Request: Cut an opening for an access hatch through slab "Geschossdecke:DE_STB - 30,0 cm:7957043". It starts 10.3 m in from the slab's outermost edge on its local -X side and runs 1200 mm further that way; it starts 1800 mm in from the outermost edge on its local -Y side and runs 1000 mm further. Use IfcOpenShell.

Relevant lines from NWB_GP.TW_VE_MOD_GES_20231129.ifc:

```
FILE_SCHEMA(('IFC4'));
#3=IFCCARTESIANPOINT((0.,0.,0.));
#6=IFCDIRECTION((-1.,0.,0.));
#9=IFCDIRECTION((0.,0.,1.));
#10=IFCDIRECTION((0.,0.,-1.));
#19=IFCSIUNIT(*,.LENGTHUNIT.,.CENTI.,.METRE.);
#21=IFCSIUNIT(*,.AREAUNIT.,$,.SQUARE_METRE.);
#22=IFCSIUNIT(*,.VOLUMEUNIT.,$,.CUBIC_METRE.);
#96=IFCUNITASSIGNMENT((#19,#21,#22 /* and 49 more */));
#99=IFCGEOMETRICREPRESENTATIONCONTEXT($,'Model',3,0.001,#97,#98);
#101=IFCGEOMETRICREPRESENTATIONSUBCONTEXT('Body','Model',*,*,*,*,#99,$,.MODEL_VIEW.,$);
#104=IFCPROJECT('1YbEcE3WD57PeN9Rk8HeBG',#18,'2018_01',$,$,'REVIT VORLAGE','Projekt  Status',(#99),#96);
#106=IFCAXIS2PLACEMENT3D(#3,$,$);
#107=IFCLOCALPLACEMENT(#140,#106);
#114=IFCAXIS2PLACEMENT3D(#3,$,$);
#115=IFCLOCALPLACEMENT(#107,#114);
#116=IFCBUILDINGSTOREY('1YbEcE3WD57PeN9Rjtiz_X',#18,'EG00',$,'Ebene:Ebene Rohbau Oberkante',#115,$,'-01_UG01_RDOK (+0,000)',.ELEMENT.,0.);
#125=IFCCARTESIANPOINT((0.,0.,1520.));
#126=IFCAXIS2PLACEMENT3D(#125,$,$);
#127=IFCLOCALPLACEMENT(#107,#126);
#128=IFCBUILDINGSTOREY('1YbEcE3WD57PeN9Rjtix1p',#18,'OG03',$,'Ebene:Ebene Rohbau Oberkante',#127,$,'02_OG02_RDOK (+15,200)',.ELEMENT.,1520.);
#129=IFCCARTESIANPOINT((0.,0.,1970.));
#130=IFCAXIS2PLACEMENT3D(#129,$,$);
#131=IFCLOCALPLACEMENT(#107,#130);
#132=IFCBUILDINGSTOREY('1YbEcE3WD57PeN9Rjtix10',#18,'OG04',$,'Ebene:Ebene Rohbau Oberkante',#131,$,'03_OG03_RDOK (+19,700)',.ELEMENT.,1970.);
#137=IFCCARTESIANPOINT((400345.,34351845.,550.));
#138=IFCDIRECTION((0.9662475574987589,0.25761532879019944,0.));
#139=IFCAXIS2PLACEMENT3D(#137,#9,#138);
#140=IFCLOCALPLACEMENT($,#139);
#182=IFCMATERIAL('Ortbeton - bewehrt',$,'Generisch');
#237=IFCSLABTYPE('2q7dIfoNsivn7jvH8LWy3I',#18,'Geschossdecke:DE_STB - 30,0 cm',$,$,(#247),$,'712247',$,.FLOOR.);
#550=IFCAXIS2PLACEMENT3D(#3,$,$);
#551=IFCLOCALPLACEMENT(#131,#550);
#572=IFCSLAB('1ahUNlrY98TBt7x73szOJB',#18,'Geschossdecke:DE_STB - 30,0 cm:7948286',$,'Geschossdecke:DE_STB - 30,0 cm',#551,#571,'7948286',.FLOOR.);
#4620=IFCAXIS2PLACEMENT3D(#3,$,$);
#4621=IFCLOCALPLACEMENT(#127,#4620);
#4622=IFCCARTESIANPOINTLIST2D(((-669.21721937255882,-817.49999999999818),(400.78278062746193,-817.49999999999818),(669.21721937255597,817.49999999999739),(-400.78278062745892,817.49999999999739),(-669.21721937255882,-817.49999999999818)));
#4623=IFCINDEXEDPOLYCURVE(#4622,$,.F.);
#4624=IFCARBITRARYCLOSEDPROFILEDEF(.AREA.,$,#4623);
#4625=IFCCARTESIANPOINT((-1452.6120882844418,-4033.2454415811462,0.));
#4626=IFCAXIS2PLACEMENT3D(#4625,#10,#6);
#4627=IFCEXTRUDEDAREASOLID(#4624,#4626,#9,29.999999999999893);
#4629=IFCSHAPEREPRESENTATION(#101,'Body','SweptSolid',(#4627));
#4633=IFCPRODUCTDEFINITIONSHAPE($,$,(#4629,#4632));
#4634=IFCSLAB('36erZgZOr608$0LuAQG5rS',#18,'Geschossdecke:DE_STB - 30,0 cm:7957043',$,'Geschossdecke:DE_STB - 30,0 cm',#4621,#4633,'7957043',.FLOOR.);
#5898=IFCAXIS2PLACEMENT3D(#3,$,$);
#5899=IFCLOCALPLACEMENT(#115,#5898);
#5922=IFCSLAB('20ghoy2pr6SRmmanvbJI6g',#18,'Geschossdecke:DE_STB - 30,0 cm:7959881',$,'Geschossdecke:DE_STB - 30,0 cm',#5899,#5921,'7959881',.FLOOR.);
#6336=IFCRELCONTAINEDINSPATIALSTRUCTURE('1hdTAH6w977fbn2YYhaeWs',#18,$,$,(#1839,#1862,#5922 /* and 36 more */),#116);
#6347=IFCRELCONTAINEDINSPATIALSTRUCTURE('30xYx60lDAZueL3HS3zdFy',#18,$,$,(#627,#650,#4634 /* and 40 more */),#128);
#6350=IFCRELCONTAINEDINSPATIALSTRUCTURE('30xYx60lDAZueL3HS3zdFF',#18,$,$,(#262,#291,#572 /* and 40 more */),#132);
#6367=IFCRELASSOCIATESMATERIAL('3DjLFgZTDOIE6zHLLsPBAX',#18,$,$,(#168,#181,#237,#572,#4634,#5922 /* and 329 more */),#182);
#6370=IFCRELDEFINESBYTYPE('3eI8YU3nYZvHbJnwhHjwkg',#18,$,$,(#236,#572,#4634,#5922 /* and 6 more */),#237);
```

```python
import numpy as np
import ifcopenshell
import ifcopenshell.api.feature
import ifcopenshell.api.geometry
import ifcopenshell.api.root
import ifcopenshell.geom
import ifcopenshell.util.placement
import ifcopenshell.util.representation
import ifcopenshell.util.shape
import ifcopenshell.util.unit

model = ifcopenshell.open("NWB_GP.TW_VE_MOD_GES_20231129.ifc")
unit_scale = ifcopenshell.util.unit.calculate_unit_scale(model)
settings = ifcopenshell.geom.settings()


def volume(element):
    """Net volume in cubic metres, openings subtracted."""
    shape = ifcopenshell.geom.create_shape(settings, element)
    return ifcopenshell.util.shape.get_volume(shape.geometry)


slab = model.by_guid("36erZgZOr608$0LuAQG5rS")
before = volume(slab)

# Extent in the slab's own axes, in metres. The edges named are its -X and -Y sides.
slab_shape = ifcopenshell.geom.create_shape(settings, slab)
vertices = ifcopenshell.util.shape.get_vertices(slab_shape.geometry)
x_min, y_min, bottom = vertices.min(axis=0)
top = vertices[:, 2].max()

opening = ifcopenshell.api.root.create_entity(model, ifc_class="IfcOpeningElement", name="Access hatch opening", predefined_type="OPENING")
context = ifcopenshell.util.representation.get_context(model, "Model", "Body", "MODEL_VIEW")
width, depth = 1.2, 1
outline = [(0.0, 0.0), (width, 0.0), (width, depth), (0.0, depth), (0.0, 0.0)]
# Overshoot both faces by 50 mm so the cut is clean.
shape = ifcopenshell.api.geometry.add_slab_representation(
    model, context=context, depth=top - bottom + 0.1, polyline=outline
)
ifcopenshell.api.geometry.assign_representation(model, product=opening, representation=shape)

matrix = ifcopenshell.util.placement.get_local_placement(slab.ObjectPlacement)
matrix[:, 3] = matrix @ np.append(np.array([x_min + 10.3, y_min + 1.8, bottom - 0.05]) / unit_scale, 1.0)
ifcopenshell.api.geometry.edit_object_placement(model, product=opening, matrix=matrix, is_si=False)
ifcopenshell.api.feature.add_feature(model, feature=opening, element=slab)

after = volume(slab)

print(f"slab volume {before:.3f} -> {after:.3f} m3")

model.write("NWB_GP.TW_VE_MOD_GES_20231129-out.ifc")
```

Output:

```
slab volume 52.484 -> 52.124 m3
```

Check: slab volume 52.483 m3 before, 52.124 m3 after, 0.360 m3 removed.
